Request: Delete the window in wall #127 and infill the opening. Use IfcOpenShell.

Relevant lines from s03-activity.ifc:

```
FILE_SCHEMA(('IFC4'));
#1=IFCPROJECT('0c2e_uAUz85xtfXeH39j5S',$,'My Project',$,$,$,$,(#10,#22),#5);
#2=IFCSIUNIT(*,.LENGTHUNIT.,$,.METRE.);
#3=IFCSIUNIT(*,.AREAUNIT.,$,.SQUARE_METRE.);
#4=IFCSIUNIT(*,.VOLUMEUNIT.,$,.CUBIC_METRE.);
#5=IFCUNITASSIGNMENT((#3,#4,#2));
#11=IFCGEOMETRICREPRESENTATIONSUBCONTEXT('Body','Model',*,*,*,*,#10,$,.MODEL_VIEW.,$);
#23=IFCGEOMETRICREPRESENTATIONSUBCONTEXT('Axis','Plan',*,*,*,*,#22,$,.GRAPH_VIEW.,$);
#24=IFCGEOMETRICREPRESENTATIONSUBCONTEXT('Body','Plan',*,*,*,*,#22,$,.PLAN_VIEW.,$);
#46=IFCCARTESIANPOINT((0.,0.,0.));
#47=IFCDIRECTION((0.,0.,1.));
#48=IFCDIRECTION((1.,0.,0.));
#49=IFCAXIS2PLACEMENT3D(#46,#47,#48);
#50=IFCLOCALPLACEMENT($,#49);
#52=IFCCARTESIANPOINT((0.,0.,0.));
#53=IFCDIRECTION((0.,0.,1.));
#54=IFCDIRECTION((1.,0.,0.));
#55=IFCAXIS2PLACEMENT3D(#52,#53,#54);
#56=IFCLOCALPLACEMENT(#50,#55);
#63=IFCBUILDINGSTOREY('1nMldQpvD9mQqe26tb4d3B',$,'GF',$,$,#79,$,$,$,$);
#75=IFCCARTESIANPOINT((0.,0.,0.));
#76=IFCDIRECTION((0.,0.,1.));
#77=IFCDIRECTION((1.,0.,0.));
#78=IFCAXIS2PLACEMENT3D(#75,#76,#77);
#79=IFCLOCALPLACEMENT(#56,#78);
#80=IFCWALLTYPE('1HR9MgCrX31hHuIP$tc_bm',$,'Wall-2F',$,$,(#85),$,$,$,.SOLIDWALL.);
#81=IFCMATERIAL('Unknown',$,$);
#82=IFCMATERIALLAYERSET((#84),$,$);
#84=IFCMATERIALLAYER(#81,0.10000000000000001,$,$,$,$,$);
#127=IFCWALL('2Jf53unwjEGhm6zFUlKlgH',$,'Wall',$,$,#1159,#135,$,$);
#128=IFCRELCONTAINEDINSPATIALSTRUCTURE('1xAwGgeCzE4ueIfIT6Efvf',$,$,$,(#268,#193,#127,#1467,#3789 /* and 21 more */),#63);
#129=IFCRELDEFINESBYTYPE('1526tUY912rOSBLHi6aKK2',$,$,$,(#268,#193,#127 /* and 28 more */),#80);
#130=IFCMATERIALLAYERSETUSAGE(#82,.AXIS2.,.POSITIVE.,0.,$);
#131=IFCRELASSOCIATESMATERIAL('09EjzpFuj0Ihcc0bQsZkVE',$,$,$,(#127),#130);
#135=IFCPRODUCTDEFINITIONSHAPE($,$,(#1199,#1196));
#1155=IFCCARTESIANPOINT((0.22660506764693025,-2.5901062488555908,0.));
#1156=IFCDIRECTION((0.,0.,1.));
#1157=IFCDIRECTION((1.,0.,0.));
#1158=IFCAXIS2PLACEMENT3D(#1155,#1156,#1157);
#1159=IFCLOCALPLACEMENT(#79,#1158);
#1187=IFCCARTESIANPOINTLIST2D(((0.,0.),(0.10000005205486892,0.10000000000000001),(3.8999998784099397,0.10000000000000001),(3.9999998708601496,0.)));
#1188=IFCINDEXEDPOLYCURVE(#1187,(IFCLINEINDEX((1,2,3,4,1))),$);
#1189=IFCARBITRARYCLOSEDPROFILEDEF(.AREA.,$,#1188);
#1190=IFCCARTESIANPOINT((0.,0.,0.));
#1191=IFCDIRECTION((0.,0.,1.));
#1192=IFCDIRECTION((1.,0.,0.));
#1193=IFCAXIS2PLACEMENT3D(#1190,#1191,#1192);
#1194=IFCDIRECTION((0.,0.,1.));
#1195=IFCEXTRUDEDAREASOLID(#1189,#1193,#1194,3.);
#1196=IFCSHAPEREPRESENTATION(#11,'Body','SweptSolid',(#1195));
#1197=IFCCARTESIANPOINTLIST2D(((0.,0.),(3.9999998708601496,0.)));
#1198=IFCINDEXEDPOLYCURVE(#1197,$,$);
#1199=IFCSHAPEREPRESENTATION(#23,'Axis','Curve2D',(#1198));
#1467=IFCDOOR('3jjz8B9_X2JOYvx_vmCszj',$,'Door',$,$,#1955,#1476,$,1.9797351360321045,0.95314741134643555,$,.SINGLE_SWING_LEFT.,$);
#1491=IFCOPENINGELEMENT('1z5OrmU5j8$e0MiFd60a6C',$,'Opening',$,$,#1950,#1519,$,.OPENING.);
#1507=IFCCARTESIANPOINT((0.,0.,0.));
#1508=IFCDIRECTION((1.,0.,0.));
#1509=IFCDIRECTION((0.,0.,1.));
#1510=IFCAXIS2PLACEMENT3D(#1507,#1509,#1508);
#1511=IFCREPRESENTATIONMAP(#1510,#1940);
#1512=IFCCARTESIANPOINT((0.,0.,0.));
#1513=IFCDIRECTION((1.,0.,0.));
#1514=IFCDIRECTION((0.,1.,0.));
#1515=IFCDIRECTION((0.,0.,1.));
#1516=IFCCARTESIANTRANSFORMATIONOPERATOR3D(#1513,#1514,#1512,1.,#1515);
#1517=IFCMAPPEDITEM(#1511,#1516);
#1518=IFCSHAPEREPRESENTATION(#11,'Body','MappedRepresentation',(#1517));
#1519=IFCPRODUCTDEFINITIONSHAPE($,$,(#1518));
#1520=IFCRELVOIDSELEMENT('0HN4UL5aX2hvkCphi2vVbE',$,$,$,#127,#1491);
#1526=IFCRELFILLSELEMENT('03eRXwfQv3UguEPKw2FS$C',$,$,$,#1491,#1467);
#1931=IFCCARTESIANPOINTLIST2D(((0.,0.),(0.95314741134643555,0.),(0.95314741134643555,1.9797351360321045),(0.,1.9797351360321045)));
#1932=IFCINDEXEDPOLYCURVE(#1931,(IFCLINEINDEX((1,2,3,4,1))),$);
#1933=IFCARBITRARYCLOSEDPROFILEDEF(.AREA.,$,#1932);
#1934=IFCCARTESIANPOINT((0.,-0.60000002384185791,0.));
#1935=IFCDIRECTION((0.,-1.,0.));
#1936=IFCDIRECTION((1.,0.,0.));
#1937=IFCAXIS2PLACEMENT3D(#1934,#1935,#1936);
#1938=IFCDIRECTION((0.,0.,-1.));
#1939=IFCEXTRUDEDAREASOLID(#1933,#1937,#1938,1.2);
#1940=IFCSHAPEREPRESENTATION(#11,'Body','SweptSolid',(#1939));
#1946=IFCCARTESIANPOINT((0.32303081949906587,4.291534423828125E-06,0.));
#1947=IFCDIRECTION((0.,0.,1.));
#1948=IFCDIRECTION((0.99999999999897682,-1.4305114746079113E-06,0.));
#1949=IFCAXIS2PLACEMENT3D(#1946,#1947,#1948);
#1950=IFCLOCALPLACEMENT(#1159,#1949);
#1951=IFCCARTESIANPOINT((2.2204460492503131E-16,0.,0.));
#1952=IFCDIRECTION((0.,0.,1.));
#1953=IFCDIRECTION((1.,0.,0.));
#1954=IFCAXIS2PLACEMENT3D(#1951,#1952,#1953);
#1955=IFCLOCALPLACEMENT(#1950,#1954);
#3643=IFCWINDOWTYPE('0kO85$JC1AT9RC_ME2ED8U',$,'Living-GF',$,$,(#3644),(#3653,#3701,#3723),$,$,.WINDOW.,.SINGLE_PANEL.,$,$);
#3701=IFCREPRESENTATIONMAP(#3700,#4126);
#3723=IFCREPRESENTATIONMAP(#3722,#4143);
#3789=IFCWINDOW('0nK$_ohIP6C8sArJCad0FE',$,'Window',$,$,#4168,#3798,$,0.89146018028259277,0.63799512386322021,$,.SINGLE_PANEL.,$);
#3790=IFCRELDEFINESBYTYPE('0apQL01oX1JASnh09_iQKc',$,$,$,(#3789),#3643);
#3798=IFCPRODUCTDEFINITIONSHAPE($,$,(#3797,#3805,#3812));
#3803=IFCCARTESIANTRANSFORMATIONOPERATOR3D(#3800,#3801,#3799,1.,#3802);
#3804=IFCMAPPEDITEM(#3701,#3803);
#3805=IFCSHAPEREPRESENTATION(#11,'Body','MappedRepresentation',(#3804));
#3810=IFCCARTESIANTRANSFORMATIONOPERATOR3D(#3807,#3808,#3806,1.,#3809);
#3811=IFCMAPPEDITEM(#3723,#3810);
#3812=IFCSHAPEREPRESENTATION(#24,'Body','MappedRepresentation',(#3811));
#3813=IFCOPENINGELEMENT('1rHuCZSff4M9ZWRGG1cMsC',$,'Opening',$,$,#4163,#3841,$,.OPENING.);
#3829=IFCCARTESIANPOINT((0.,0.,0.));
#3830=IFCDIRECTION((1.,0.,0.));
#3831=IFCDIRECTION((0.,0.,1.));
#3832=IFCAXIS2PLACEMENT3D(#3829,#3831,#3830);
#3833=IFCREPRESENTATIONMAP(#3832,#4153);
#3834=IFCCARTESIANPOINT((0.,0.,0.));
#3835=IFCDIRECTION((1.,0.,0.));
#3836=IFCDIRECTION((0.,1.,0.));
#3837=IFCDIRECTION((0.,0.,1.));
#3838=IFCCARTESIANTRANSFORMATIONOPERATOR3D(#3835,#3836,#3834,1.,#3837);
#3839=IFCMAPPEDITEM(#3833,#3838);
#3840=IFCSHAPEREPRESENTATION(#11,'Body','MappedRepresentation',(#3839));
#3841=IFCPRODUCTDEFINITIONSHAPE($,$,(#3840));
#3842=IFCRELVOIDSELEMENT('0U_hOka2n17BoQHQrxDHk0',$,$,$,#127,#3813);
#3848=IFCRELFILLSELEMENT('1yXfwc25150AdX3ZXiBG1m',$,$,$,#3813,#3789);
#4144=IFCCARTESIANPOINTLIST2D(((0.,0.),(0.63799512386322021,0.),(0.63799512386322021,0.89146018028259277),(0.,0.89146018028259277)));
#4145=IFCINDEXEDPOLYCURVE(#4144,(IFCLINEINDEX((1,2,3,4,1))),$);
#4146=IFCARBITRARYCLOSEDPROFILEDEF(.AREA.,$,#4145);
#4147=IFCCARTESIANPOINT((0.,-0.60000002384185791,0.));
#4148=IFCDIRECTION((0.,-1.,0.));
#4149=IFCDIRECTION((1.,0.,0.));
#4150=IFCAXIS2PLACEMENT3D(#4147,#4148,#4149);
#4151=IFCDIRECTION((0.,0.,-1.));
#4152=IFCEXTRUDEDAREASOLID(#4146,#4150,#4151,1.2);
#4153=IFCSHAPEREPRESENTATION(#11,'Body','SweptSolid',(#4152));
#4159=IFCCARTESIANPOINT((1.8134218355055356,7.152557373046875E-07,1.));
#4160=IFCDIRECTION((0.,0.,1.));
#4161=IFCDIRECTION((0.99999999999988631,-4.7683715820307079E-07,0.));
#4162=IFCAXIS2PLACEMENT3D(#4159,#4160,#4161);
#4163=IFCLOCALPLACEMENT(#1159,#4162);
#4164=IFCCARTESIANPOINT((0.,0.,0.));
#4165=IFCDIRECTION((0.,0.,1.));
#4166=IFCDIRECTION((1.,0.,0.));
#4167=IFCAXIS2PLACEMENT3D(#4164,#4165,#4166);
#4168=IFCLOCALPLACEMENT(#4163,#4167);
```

```python
import ifcopenshell
import ifcopenshell.api.feature
import ifcopenshell.api.root
import ifcopenshell.geom
import ifcopenshell.util.shape

model = ifcopenshell.open("s03-activity.ifc")
settings = ifcopenshell.geom.settings()


def volume(element):
    """Net volume in cubic metres, openings subtracted."""
    shape = ifcopenshell.geom.create_shape(settings, element)
    return ifcopenshell.util.shape.get_volume(shape.geometry)


window = model.by_guid("0nK$_ohIP6C8sArJCad0FE")
opening = window.FillsVoids[0].RelatingOpeningElement
wall = opening.VoidsElements[0].RelatingBuildingElement
before = volume(wall)

ifcopenshell.api.root.remove_product(model, product=window)
ifcopenshell.api.feature.remove_feature(model, feature=opening)

after = volume(wall)

print(f"wall volume {before:.3f} -> {after:.3f} m3")

model.write("s03-activity_edited.ifc")
```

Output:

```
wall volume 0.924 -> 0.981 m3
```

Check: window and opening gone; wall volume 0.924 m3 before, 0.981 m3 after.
